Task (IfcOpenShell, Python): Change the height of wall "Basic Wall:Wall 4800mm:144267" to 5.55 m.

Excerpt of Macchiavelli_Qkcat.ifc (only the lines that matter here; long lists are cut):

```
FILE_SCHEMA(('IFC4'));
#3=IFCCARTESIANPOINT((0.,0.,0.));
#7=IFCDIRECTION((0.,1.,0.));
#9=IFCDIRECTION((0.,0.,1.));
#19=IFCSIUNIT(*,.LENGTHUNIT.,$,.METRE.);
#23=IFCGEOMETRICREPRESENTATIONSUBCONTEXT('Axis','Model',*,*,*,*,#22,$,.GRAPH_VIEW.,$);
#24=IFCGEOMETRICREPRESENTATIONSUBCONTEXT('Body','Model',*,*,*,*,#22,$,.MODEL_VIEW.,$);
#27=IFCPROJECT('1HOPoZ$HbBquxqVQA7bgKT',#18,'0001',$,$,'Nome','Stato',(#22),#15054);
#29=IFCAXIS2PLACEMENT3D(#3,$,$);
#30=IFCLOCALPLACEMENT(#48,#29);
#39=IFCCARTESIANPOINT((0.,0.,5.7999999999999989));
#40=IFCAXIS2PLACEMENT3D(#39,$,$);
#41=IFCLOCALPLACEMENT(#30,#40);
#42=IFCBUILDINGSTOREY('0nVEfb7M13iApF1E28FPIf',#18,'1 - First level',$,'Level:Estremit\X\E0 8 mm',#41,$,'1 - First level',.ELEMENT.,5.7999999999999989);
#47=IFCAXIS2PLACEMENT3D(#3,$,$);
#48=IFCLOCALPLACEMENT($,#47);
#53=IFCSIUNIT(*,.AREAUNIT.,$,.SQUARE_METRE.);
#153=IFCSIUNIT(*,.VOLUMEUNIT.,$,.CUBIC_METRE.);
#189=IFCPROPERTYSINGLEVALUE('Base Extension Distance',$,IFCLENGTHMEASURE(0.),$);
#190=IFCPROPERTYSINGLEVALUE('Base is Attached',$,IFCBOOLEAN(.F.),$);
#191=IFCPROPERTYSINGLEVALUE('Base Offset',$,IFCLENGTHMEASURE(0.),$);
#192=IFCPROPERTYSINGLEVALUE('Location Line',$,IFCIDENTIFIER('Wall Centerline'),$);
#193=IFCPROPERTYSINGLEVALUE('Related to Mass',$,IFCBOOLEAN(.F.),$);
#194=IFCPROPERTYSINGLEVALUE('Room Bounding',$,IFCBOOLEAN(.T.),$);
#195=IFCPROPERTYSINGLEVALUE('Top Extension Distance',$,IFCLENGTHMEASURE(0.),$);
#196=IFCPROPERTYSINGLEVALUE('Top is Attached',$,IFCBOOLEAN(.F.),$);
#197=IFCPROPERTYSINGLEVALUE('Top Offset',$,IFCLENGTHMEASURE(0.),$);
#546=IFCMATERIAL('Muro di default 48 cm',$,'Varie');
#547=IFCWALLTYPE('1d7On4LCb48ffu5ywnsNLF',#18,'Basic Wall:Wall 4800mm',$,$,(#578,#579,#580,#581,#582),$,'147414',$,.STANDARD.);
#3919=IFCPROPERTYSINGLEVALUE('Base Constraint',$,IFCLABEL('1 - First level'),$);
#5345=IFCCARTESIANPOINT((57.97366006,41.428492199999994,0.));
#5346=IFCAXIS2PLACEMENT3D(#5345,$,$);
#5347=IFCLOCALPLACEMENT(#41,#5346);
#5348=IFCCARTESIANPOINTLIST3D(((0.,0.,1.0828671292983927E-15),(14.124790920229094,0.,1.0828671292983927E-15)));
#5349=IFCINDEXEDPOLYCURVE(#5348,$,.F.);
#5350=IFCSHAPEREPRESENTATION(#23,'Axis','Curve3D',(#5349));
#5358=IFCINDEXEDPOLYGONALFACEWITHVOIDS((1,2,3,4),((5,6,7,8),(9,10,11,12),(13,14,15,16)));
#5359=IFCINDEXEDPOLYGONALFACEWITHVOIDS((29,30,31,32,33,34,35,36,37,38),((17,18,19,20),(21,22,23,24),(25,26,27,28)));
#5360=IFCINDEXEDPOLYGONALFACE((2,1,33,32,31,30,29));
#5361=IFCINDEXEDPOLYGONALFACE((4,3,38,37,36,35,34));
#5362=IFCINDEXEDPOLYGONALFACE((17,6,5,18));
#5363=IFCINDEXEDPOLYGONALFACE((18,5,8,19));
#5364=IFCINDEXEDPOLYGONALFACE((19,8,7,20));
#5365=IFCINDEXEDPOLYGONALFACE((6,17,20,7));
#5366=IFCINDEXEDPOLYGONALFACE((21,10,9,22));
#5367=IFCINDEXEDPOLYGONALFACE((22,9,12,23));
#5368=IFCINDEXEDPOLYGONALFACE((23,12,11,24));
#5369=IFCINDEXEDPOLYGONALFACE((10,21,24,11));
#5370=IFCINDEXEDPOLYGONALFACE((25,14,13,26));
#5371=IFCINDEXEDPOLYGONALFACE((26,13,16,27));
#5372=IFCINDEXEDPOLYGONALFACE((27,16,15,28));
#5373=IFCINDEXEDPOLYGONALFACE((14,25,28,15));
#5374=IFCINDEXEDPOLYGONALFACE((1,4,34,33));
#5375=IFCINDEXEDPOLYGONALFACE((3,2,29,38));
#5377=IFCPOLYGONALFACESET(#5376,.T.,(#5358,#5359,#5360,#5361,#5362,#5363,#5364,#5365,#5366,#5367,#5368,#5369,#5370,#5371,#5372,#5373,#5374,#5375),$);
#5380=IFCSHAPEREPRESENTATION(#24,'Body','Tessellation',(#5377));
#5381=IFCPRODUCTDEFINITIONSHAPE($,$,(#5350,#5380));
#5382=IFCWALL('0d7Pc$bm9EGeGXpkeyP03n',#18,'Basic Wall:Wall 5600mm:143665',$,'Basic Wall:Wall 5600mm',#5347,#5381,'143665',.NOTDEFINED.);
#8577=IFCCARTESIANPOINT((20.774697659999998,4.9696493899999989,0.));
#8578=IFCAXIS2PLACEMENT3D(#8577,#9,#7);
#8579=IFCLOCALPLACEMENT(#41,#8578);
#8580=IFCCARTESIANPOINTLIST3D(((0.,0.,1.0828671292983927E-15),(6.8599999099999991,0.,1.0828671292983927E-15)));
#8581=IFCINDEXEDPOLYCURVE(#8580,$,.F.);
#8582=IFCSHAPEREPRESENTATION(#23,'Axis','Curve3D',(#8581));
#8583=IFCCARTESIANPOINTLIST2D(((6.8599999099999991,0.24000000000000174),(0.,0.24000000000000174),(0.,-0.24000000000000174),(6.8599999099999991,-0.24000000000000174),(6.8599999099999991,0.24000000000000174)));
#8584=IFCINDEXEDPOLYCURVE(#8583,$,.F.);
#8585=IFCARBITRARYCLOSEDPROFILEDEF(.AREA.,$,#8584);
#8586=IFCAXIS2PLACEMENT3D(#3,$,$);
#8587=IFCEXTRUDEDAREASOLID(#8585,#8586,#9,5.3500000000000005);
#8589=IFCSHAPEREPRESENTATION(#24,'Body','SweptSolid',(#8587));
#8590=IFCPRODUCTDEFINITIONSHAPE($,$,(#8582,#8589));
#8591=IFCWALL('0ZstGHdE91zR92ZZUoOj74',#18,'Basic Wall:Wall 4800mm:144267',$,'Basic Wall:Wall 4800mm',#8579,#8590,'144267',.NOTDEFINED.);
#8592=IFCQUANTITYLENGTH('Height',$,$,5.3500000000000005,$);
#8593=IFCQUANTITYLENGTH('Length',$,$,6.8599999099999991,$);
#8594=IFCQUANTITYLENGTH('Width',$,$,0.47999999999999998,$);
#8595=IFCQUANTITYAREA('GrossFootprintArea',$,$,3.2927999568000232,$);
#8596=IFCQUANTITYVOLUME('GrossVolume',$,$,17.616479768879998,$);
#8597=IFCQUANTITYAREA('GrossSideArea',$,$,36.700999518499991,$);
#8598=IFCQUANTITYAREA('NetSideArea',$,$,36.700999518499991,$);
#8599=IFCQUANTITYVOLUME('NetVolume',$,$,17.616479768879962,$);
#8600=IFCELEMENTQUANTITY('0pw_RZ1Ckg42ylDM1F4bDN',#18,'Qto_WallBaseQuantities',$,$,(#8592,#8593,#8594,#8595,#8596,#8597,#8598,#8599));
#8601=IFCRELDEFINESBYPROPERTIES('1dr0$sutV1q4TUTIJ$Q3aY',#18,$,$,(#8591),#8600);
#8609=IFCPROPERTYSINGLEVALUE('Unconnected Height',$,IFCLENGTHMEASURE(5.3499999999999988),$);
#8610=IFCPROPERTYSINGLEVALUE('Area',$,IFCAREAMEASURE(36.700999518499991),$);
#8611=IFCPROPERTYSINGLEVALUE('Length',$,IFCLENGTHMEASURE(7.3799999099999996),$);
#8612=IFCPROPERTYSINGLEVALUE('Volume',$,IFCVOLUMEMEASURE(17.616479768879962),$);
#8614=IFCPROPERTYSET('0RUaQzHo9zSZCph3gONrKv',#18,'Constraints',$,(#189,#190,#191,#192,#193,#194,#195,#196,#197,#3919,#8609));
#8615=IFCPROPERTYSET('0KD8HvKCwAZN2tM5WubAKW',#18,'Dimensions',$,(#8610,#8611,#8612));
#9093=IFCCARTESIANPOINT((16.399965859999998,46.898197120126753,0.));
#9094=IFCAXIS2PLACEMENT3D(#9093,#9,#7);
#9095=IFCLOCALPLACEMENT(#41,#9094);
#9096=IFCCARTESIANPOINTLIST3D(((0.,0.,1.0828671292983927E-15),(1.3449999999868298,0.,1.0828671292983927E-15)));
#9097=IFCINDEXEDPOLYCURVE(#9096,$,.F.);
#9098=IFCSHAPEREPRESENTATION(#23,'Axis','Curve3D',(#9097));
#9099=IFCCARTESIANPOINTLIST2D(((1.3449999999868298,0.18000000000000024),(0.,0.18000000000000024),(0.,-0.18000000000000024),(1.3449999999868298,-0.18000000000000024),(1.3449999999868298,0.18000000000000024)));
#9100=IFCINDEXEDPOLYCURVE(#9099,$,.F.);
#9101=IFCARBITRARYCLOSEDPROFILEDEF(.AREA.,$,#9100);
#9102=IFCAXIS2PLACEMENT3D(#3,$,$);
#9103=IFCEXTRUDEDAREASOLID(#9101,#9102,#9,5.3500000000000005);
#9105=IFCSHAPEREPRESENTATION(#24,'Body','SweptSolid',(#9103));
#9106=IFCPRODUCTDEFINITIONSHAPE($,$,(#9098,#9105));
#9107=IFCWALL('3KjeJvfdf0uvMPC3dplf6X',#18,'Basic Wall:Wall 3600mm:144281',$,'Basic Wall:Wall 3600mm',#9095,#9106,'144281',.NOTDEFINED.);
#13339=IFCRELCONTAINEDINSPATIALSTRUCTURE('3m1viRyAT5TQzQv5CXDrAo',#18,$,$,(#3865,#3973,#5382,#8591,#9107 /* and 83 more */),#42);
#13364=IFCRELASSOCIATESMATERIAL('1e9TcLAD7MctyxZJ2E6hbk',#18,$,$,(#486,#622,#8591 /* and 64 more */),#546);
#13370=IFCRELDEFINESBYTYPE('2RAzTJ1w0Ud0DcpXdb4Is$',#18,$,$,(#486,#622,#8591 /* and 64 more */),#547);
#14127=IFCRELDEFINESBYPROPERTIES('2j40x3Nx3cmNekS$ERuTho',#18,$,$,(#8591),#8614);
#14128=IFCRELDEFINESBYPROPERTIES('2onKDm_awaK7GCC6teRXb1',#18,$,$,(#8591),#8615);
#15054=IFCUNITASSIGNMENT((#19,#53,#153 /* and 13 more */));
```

```python
import ifcopenshell
import ifcopenshell.api.pset
import ifcopenshell.geom
import ifcopenshell.util.element
import ifcopenshell.util.representation
import ifcopenshell.util.shape
import ifcopenshell.util.unit

model = ifcopenshell.open("Macchiavelli_Qkcat.ifc")
unit_scale = ifcopenshell.util.unit.calculate_unit_scale(model)
area_scale = ifcopenshell.util.unit.calculate_unit_scale(model, "AREAUNIT")
volume_scale = ifcopenshell.util.unit.calculate_unit_scale(model, "VOLUMEUNIT")
settings = ifcopenshell.geom.settings()


def volume(element):
    """Net volume in cubic metres, openings subtracted."""
    shape = ifcopenshell.geom.create_shape(settings, element)
    return ifcopenshell.util.shape.get_volume(shape.geometry)


wall = model.by_id(8591)
before = volume(wall)

body = ifcopenshell.util.representation.get_representation(wall, "Model", "Body")
solid = body.Items[0]
old_height = solid.Depth
solid.Depth = 5.55 / unit_scale
after = volume(wall)
thickness = 0.48  # wall thickness in metres

# Update the stored height, areas and volumes.
qto = model.by_id(ifcopenshell.util.element.get_pset(wall, "Qto_WallBaseQuantities", should_inherit=False)["id"])
ifcopenshell.api.pset.edit_qto(model, qto=qto, properties={
    "Height": solid.Depth,
    "GrossVolume": ifcopenshell.util.element.get_pset(wall, "Qto_WallBaseQuantities", "GrossVolume") * solid.Depth / old_height,
    "GrossSideArea": ifcopenshell.util.element.get_pset(wall, "Qto_WallBaseQuantities", "GrossSideArea") * solid.Depth / old_height,
    "NetSideArea": after / thickness / area_scale,
    "NetVolume": after / volume_scale,
})
pset = model.by_id(ifcopenshell.util.element.get_pset(wall, "Constraints", should_inherit=False)["id"])
ifcopenshell.api.pset.edit_pset(model, pset=pset, properties={
    "Unconnected Height": model.create_entity("IfcLengthMeasure", solid.Depth),
})
pset = model.by_id(ifcopenshell.util.element.get_pset(wall, "Dimensions", should_inherit=False)["id"])
ifcopenshell.api.pset.edit_pset(model, pset=pset, properties={
    "Area": model.create_entity("IfcAreaMeasure", after / thickness / area_scale),
    "Volume": model.create_entity("IfcVolumeMeasure", after / volume_scale),
})

print(f"height {old_height:g} -> {solid.Depth:g}, volume {before:.3f} -> {after:.3f} m3")

model.write("Macchiavelli_Qkcat_v2.ifc")
```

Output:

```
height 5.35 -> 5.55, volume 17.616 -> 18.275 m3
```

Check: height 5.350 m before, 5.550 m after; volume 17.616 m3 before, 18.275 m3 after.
